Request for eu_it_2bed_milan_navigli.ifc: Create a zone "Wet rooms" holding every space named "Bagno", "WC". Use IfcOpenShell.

First a look at what the model holds.

```python
import ifcopenshell

model = ifcopenshell.open("eu_it_2bed_milan_navigli.ifc")
print(model.schema)
seen = {}
for space in model.by_type("IfcSpace"):
    seen[space.LongName] = seen.get(space.LongName, 0) + 1
for name, count in sorted(seen.items(), key=str):
    print(count, "x", name)
print("zones:", [z.Name for z in model.by_type("IfcZone")][:20])
```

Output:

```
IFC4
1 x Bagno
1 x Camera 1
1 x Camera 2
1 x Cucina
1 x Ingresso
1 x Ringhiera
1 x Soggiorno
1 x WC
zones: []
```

```python
import ifcopenshell
import ifcopenshell.api.group
import ifcopenshell.api.root

model = ifcopenshell.open("eu_it_2bed_milan_navigli.ifc")

names = {"Bagno", "WC"}
spaces = [s for s in model.by_type("IfcSpace") if s.LongName in names]

zone = ifcopenshell.api.root.create_entity(model, ifc_class="IfcZone", name="Wet rooms")
ifcopenshell.api.group.assign_group(model, products=spaces, group=zone)
print(len(spaces), "spaces in", zone.Name)

model.write("eu_it_2bed_milan_navigli_v2.ifc")
```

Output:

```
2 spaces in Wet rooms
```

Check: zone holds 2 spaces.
